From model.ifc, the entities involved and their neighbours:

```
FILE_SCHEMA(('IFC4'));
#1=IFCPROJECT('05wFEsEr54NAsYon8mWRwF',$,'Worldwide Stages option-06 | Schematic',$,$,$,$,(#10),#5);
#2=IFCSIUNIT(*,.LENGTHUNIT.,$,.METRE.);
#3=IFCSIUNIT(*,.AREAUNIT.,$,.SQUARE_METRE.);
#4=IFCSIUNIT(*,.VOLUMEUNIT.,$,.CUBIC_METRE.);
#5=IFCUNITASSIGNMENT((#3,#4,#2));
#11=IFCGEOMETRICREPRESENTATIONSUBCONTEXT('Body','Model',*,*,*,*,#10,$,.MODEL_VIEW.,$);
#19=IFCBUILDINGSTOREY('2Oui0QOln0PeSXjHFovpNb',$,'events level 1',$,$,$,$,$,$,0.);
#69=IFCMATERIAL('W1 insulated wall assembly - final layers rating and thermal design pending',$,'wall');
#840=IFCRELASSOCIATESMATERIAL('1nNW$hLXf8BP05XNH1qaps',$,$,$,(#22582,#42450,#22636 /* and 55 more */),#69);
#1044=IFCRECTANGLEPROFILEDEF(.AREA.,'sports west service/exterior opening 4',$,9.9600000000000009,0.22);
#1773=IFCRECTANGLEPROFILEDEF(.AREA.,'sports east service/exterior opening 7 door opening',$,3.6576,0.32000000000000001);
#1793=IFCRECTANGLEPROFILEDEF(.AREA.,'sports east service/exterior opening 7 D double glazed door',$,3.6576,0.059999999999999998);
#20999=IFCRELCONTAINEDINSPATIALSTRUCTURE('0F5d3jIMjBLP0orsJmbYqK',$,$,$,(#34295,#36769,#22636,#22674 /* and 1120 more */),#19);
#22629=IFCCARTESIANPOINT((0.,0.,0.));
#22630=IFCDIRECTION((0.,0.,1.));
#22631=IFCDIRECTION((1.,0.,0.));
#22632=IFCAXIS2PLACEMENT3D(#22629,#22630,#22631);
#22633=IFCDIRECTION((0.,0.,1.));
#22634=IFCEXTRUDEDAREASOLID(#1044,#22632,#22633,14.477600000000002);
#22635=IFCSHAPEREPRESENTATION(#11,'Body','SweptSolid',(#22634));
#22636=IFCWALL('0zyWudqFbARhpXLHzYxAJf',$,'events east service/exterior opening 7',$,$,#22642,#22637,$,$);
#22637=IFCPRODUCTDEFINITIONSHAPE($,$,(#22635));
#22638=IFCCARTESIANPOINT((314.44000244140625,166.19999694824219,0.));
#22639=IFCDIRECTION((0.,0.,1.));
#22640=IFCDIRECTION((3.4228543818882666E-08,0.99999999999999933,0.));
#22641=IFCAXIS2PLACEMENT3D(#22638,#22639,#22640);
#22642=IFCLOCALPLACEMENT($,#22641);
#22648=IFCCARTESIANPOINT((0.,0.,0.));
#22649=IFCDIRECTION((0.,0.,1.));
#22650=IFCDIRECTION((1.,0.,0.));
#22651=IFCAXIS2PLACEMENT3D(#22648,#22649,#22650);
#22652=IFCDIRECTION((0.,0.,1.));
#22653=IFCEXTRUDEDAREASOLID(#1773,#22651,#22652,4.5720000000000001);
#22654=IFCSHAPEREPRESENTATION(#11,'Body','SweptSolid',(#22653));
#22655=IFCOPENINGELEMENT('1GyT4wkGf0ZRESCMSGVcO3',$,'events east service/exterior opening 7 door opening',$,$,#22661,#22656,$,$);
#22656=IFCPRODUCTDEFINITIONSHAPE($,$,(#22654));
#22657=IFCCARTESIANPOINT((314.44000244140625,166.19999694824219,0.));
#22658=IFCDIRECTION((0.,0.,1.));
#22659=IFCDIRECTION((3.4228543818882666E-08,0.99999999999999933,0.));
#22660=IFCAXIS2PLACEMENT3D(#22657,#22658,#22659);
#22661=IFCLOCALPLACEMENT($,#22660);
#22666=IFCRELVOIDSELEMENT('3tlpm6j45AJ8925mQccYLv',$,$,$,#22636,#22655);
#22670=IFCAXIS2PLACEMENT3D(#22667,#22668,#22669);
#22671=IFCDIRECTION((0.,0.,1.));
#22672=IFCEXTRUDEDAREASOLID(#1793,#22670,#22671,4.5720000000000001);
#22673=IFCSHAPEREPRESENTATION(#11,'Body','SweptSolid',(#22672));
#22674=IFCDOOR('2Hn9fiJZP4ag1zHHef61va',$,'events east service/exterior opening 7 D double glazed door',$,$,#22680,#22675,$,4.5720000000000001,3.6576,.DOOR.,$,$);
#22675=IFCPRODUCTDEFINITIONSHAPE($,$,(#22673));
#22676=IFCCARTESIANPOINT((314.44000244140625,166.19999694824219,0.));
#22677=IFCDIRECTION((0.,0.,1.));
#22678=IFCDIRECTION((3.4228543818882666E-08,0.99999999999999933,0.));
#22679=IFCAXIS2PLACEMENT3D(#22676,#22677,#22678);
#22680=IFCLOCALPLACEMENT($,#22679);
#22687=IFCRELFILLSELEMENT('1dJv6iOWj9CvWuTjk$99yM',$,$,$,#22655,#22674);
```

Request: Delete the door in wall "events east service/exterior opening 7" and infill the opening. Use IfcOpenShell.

```python
import ifcopenshell
import ifcopenshell.api.feature
import ifcopenshell.api.root
import ifcopenshell.geom
import ifcopenshell.util.shape

model = ifcopenshell.open("model.ifc")
settings = ifcopenshell.geom.settings()


def volume(element):
    """Net volume in cubic metres, openings subtracted."""
    shape = ifcopenshell.geom.create_shape(settings, element)
    return ifcopenshell.util.shape.get_volume(shape.geometry)


door = model.by_id(22674)
opening = door.FillsVoids[0].RelatingOpeningElement
wall = opening.VoidsElements[0].RelatingBuildingElement
before = volume(wall)

ifcopenshell.api.root.remove_product(model, product=door)
ifcopenshell.api.feature.remove_feature(model, feature=opening)

after = volume(wall)

print(f"wall volume {before:.3f} -> {after:.3f} m3")

model.write("model_rev.ifc")
```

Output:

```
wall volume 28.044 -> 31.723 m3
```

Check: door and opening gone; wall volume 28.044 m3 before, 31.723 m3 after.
